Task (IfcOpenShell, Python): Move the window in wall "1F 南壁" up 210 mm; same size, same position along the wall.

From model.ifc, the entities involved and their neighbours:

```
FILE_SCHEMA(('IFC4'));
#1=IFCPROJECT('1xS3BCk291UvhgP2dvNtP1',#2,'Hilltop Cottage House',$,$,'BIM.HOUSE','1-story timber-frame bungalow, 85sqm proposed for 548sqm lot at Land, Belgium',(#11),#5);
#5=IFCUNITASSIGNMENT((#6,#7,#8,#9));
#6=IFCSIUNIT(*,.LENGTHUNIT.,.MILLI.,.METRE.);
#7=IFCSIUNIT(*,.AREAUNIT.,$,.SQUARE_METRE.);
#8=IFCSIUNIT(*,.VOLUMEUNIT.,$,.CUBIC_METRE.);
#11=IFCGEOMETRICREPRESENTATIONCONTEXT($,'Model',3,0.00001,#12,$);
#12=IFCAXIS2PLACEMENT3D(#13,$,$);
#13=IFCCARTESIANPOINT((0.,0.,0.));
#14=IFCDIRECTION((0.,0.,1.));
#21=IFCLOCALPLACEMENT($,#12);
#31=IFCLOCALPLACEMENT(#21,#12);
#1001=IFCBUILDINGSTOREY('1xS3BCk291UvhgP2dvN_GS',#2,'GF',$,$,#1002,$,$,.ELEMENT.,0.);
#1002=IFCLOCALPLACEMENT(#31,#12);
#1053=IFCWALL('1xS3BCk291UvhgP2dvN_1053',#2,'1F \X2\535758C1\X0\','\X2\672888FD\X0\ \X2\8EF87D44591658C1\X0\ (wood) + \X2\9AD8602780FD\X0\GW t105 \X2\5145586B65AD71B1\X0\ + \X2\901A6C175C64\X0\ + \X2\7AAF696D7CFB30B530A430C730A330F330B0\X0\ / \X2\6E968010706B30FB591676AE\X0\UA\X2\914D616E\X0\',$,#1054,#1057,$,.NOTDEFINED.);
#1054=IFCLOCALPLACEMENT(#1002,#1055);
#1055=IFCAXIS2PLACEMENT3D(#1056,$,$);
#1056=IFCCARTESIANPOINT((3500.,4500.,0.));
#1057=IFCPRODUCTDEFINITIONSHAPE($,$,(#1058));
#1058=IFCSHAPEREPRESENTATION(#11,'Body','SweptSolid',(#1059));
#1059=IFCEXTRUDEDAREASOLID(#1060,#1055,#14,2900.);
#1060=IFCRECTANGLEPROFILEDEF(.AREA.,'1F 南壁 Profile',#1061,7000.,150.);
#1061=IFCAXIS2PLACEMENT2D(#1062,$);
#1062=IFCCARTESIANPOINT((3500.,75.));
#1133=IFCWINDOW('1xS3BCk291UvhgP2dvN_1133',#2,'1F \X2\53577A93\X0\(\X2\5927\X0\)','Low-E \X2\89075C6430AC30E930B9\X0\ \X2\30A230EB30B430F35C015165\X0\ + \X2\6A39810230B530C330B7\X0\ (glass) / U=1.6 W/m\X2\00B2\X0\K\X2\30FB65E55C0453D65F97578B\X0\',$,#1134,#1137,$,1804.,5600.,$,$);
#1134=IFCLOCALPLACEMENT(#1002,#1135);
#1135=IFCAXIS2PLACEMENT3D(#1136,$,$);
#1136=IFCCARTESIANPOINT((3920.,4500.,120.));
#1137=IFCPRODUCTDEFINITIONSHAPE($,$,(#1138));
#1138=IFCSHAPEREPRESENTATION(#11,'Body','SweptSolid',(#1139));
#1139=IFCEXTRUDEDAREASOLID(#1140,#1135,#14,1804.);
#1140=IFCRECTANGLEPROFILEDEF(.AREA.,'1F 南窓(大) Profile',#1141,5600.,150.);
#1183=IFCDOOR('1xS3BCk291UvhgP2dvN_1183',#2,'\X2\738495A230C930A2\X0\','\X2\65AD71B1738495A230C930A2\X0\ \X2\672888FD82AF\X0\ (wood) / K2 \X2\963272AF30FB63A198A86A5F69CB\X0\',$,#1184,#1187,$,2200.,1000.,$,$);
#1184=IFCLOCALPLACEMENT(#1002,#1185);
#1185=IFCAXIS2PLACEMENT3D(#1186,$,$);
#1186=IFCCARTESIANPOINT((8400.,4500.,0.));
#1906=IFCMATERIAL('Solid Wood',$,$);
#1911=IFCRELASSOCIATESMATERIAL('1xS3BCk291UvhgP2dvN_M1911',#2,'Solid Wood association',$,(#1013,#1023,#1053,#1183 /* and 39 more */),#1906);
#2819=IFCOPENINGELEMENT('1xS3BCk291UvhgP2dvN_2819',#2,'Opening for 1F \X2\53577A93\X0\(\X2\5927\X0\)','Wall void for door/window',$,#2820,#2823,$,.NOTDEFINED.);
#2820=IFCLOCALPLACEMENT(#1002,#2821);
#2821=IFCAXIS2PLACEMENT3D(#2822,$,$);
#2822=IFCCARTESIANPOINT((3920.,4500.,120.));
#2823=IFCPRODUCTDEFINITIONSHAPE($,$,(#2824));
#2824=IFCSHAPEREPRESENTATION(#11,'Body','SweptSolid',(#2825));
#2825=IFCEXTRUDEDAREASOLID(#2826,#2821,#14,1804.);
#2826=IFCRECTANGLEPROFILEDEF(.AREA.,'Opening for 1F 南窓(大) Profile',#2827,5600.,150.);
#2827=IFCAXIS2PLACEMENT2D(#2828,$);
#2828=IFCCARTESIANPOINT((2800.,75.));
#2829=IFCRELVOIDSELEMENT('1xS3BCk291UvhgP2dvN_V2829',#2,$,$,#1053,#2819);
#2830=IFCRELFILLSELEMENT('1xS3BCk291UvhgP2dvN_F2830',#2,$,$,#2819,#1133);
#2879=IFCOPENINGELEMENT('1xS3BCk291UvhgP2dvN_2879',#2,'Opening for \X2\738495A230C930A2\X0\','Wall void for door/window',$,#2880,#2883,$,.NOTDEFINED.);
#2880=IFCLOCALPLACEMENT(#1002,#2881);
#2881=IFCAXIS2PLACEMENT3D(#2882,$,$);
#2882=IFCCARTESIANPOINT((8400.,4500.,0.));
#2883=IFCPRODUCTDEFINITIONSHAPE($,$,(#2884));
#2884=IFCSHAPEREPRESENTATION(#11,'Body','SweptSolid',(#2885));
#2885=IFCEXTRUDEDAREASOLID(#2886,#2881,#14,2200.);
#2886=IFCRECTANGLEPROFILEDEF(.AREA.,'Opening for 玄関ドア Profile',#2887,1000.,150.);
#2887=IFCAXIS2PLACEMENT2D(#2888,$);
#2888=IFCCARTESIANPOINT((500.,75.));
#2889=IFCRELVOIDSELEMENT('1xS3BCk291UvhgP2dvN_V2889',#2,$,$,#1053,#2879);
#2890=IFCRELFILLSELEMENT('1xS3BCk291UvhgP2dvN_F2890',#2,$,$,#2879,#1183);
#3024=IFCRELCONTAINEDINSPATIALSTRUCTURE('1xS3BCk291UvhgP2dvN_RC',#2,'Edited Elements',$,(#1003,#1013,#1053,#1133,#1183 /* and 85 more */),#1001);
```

```python
import numpy as np
import ifcopenshell
import ifcopenshell.api.geometry
import ifcopenshell.util.placement
import ifcopenshell.util.unit

model = ifcopenshell.open("model.ifc")
unit_scale = ifcopenshell.util.unit.calculate_unit_scale(model)

window = model.by_guid("1xS3BCk291UvhgP2dvN_1133")
opening = window.FillsVoids[0].RelatingOpeningElement
dz = 210.0

shift = np.array([0.0, 0.0, dz])
# The window is not placed relative to its opening, so move both.
for product in (opening, window):
    matrix = ifcopenshell.util.placement.get_local_placement(product.ObjectPlacement)
    matrix[:3, 3] += shift
    ifcopenshell.api.geometry.edit_object_placement(model, product=product, matrix=matrix, is_si=False)

print(f"moved by {dz * unit_scale:+.3f} m")

model.write("model_updated.ifc")
```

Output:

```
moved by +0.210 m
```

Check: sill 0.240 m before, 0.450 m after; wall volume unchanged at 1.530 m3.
